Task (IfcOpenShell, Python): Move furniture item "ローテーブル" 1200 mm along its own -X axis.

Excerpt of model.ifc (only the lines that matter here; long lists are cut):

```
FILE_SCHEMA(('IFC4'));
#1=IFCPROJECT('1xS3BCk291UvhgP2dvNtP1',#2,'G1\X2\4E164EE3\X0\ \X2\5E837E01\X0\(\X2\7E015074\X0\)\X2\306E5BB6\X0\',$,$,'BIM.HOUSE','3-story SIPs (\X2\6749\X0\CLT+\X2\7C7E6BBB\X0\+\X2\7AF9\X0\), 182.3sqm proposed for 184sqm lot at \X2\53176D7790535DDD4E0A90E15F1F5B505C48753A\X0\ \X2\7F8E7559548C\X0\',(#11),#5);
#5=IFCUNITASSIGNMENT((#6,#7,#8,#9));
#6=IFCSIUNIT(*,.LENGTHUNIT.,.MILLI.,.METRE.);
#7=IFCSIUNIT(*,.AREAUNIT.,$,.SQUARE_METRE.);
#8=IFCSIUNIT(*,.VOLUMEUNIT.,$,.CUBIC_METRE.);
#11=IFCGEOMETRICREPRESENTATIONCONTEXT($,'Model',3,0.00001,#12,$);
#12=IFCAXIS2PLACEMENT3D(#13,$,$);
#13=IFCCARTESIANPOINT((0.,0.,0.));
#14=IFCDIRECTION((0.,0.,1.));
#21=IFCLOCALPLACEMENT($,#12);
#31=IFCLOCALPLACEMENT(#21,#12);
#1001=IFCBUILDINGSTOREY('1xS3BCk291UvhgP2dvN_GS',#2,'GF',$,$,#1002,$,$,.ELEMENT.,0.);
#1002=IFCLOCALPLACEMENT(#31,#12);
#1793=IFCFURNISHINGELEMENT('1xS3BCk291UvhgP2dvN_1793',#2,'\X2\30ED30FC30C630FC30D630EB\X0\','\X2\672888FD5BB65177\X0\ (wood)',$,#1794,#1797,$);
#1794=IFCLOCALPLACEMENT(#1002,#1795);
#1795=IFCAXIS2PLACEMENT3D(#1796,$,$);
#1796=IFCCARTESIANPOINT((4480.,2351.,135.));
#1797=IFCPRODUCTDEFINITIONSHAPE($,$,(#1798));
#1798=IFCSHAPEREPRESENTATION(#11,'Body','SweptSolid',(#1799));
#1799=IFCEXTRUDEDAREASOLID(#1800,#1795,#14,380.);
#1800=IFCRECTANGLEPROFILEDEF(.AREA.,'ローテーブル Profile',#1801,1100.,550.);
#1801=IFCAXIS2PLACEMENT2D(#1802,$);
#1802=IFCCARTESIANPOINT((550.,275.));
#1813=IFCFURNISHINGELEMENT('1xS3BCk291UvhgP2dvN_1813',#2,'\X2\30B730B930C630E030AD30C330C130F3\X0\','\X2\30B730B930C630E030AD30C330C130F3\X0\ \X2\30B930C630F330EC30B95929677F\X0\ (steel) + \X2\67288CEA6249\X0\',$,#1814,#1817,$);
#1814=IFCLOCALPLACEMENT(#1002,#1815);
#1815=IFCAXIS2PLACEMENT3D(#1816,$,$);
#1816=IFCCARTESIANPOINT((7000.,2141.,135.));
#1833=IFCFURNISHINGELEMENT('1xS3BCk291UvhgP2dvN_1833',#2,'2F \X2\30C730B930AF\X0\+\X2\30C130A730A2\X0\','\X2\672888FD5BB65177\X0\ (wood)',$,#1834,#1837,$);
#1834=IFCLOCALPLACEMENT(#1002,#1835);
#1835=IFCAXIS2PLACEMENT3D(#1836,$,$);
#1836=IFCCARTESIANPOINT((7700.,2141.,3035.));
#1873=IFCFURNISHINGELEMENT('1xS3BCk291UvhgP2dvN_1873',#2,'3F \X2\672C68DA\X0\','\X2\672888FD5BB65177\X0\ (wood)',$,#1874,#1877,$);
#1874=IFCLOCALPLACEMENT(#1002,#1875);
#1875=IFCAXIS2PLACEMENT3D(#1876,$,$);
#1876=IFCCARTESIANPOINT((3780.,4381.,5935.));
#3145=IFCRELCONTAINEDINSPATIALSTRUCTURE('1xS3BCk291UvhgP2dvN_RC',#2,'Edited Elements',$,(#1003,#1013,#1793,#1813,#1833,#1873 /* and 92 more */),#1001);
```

```python
import ifcopenshell
import ifcopenshell.api.geometry
import ifcopenshell.util.placement

model = ifcopenshell.open("model.ifc")

item = model.by_guid("1xS3BCk291UvhgP2dvN_1793")
matrix = ifcopenshell.util.placement.get_local_placement(item.ObjectPlacement)
matrix[:3, 3] -= matrix[:3, 0] * 1200.0
ifcopenshell.api.geometry.edit_object_placement(model, product=item, matrix=matrix, is_si=False)

print(ifcopenshell.util.placement.get_local_placement(item.ObjectPlacement).round(3) + 0.0)

model.write("model_edited.ifc")
```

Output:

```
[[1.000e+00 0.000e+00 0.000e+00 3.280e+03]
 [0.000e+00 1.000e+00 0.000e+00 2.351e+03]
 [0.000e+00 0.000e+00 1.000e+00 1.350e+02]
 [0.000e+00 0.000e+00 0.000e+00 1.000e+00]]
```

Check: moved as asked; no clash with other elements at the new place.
